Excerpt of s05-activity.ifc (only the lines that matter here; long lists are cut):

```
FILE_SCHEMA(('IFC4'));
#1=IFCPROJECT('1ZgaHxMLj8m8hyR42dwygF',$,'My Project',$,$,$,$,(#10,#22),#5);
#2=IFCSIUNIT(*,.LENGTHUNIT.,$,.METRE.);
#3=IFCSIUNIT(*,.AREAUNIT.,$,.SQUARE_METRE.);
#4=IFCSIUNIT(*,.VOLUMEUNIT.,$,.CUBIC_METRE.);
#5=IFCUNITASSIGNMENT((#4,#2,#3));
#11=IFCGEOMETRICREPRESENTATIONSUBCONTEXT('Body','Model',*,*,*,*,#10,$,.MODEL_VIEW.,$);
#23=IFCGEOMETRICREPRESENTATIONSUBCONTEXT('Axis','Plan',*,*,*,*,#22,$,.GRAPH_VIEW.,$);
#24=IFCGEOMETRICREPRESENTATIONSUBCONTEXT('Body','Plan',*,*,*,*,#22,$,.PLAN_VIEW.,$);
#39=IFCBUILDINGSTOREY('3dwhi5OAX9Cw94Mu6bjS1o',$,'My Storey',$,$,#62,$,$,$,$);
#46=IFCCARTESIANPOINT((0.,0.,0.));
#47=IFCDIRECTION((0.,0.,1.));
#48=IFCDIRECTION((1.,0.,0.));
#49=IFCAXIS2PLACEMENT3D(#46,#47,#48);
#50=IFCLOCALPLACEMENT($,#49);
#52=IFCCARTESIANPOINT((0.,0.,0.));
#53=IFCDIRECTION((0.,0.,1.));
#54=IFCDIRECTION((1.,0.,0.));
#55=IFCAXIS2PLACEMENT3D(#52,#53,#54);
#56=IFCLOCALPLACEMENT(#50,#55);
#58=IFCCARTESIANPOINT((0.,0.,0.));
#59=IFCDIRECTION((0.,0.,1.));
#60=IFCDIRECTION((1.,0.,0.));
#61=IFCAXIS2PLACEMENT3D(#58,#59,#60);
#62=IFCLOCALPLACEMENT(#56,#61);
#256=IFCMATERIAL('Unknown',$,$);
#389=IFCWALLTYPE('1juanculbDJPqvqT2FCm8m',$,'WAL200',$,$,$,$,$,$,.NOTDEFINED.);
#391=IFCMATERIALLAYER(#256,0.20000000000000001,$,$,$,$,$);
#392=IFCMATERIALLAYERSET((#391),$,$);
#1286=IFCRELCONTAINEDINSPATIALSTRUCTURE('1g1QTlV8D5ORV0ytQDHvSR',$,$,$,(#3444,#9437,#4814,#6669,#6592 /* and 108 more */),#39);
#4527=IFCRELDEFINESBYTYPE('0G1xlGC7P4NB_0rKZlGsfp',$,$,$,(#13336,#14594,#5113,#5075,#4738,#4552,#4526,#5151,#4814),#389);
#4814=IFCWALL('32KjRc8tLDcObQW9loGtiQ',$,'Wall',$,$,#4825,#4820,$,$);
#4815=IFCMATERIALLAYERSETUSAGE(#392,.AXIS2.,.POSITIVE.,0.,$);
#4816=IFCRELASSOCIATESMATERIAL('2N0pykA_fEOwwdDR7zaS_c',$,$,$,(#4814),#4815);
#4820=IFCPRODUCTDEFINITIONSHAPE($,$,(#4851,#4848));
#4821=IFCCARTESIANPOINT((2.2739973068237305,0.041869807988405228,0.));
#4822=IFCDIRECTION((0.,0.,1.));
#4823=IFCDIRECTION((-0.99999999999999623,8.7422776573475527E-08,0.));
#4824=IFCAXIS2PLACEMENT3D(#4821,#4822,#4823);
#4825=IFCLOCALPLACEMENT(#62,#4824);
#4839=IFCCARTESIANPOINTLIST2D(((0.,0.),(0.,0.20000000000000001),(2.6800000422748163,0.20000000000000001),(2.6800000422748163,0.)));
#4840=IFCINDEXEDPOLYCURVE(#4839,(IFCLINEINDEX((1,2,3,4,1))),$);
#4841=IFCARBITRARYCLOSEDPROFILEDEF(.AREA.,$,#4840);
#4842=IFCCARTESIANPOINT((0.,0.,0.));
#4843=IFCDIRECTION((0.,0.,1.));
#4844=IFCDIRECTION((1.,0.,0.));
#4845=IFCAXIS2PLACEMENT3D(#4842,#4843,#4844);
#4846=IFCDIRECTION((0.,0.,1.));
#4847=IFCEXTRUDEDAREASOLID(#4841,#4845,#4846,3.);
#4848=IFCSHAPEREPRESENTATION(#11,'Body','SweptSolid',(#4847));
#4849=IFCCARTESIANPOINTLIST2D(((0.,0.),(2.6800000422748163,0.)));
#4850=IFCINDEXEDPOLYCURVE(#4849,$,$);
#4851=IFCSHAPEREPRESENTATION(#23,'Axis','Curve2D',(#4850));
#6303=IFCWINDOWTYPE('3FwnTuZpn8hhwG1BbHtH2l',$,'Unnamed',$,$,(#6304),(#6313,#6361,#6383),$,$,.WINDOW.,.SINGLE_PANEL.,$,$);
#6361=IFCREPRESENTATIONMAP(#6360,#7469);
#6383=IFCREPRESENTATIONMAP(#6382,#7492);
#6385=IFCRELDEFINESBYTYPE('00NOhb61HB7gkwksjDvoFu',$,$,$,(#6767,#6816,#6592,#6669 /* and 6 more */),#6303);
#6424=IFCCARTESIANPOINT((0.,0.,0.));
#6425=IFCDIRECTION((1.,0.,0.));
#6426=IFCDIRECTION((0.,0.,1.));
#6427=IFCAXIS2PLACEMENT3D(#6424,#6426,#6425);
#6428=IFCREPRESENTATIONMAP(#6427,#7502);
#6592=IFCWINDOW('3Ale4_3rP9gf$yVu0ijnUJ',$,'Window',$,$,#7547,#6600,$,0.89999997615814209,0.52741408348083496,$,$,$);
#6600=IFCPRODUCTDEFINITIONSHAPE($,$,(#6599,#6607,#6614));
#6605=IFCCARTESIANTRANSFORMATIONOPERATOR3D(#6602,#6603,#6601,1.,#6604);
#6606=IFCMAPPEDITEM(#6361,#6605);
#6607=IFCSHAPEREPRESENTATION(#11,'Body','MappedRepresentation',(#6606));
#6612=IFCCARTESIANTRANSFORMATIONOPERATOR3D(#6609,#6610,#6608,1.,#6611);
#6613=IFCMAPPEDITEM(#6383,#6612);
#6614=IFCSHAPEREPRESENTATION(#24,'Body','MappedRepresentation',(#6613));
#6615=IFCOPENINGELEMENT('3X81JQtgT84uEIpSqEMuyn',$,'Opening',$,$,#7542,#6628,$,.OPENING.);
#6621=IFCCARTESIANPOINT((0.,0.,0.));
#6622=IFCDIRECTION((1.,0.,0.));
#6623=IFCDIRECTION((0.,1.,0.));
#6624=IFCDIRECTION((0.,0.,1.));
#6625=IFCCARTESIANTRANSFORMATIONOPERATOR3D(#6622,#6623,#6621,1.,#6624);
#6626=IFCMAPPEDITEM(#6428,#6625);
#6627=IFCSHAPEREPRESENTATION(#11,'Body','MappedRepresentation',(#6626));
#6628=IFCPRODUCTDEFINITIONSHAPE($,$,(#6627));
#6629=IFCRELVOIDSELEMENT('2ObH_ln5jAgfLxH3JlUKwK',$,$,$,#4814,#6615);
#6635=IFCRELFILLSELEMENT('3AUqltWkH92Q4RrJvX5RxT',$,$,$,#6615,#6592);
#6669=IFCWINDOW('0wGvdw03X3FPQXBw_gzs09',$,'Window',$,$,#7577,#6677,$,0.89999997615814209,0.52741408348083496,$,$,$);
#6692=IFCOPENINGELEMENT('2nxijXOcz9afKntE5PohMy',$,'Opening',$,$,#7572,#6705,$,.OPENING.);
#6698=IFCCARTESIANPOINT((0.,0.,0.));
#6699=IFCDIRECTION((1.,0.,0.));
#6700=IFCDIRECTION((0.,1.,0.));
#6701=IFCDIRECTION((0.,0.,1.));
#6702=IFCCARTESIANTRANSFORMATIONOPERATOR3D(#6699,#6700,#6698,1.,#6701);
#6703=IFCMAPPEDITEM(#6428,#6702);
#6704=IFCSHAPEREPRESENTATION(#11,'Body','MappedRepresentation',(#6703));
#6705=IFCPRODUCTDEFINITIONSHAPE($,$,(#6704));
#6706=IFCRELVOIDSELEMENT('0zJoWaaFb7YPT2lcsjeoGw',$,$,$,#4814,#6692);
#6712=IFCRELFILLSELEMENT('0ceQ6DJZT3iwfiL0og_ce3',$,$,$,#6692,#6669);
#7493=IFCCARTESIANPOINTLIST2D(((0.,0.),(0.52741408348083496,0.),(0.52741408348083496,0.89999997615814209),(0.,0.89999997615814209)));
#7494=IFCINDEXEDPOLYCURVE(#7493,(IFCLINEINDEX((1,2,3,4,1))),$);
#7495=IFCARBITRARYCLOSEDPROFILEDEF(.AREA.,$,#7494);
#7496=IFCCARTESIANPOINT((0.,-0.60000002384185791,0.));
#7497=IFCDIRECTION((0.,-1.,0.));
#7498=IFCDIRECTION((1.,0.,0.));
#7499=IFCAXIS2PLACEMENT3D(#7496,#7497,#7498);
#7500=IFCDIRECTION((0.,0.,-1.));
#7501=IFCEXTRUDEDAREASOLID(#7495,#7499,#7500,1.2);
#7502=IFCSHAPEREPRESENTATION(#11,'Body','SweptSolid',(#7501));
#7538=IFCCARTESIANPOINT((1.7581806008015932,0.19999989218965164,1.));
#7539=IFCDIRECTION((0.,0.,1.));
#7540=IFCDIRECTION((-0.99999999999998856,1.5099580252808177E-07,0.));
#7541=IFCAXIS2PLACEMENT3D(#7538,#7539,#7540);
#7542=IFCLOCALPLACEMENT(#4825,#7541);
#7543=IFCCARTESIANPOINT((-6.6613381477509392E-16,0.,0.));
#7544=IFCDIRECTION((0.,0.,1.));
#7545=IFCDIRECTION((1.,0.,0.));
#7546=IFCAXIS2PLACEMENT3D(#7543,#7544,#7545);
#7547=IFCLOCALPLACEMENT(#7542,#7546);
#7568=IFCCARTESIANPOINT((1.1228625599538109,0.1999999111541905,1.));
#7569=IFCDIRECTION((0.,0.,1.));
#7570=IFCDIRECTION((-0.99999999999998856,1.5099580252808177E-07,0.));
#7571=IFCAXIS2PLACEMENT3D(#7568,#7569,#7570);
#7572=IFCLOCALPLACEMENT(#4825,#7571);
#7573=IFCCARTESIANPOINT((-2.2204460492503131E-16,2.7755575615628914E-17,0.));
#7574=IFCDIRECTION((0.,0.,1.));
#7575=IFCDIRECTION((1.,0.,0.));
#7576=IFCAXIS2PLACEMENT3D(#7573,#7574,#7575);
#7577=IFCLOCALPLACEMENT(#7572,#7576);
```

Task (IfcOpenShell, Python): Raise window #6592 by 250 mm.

```python
import numpy as np
import ifcopenshell
import ifcopenshell.api.geometry
import ifcopenshell.util.placement
import ifcopenshell.util.unit

model = ifcopenshell.open("s05-activity.ifc")
unit_scale = ifcopenshell.util.unit.calculate_unit_scale(model)

window = model.by_guid("3Ale4_3rP9gf$yVu0ijnUJ")
opening = window.FillsVoids[0].RelatingOpeningElement
dz = 0.25 / unit_scale

shift = np.array([0.0, 0.0, dz])
# The window is placed relative to its opening, so it follows when the opening moves.
matrix = ifcopenshell.util.placement.get_local_placement(opening.ObjectPlacement)
matrix[:3, 3] += shift
ifcopenshell.api.geometry.edit_object_placement(
    model, product=opening, matrix=matrix, is_si=False, should_transform_children=True
)

print(f"moved by {dz * unit_scale:+.3f} m")

model.write("s05-activity_updated.ifc")
```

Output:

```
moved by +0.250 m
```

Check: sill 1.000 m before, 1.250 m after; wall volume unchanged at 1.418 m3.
